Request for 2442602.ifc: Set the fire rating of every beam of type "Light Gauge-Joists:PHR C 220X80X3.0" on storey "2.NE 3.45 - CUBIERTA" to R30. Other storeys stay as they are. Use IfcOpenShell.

First a look at what the model holds.

```python
import ifcopenshell
import ifcopenshell.util.element

model = ifcopenshell.open("2442602.ifc")
print(model.schema)
storey = next(s for s in model.by_type("IfcBuildingStorey") if s.Name == "2.NE 3.45 - CUBIERTA")
beams = [e for e in ifcopenshell.util.element.get_decomposition(storey) if e.is_a("IfcBeam")]
seen = {}
for e in beams:
    element_type = ifcopenshell.util.element.get_type(e)
    key = (element_type.Name if element_type != e and element_type else None, ifcopenshell.util.element.get_pset(e, "Pset_BeamCommon", "FireRating"))
    seen[key] = seen.get(key, 0) + 1
for (name, value), count in sorted(seen.items(), key=str):
    print(count, "x", name, "|", value)
```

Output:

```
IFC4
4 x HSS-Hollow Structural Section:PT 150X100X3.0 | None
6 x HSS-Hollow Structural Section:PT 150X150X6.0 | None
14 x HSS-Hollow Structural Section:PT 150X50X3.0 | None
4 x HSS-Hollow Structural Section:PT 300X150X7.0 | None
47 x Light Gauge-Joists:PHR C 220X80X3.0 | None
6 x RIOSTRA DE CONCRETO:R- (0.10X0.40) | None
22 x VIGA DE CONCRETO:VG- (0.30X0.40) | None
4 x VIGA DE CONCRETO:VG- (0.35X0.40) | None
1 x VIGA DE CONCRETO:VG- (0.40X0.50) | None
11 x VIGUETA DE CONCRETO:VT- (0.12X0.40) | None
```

```python
import ifcopenshell
import ifcopenshell.api.pset
import ifcopenshell.util.element

model = ifcopenshell.open("2442602.ifc")

storey = next(s for s in model.by_type("IfcBuildingStorey") if s.Name == "2.NE 3.45 - CUBIERTA")
beams = [e for e in ifcopenshell.util.element.get_decomposition(storey) if e.is_a("IfcBeam")]

count = 0
for e in beams:
    element_type = ifcopenshell.util.element.get_type(e)
    if element_type in (None, e) or element_type.Name != "Light Gauge-Joists:PHR C 220X80X3.0":
        continue
    # add_pset returns the element's existing set when there is one.
    pset = ifcopenshell.api.pset.add_pset(model, product=e, name="Pset_BeamCommon")
    ifcopenshell.api.pset.edit_pset(model, pset=pset, properties={"FireRating": "R30"})
    count += 1

print(count, "beams updated")

model.write("2442602-out.ifc")
```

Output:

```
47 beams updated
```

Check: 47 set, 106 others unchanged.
